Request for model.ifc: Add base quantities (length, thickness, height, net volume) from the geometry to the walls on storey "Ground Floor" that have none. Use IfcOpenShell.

First a look at what the model holds.

```python
import ifcopenshell
import ifcopenshell.util.element
import ifcopenshell.util.unit

model = ifcopenshell.open("model.ifc")
print(model.schema)
for unit_type in ("LENGTHUNIT", "AREAUNIT", "VOLUMEUNIT"):
    print(unit_type, ifcopenshell.util.unit.calculate_unit_scale(model, unit_type))
storey = next(s for s in model.by_type("IfcBuildingStorey") if s.Name == "Ground Floor")
walls = [e for e in ifcopenshell.util.element.get_decomposition(storey) if e.is_a("IfcWall")]
for e in sorted(walls, key=lambda e: e.id()):
    print(e.id(), e.is_a(), e.Name, list(ifcopenshell.util.element.get_psets(e, qtos_only=True)), sep=" | ")
```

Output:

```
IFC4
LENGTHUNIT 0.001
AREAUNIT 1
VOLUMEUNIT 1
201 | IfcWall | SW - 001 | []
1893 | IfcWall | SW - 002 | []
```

```python
import ifcopenshell
import ifcopenshell.api.pset
import ifcopenshell.geom
import ifcopenshell.util.element
import ifcopenshell.util.shape
import ifcopenshell.util.unit

model = ifcopenshell.open("model.ifc")
unit_scale = ifcopenshell.util.unit.calculate_unit_scale(model)
volume_scale = ifcopenshell.util.unit.calculate_unit_scale(model, "VOLUMEUNIT")
settings = ifcopenshell.geom.settings()

storey = next(s for s in model.by_type("IfcBuildingStorey") if s.Name == "Ground Floor")
walls = [e for e in ifcopenshell.util.element.get_decomposition(storey) if e.is_a("IfcWall")]

for e in sorted(walls, key=lambda e: e.id()):
    if ifcopenshell.util.element.get_psets(e, qtos_only=True, should_inherit=False):
        continue
    # Geometry comes back in metres, in the element's own axes.
    shape = ifcopenshell.geom.create_shape(settings, e)
    values = {
        "Length": ifcopenshell.util.shape.get_x(shape.geometry) / unit_scale,
        "Width": ifcopenshell.util.shape.get_y(shape.geometry) / unit_scale,
        "Height": ifcopenshell.util.shape.get_z(shape.geometry) / unit_scale,
        "NetVolume": ifcopenshell.util.shape.get_volume(shape.geometry) / volume_scale,
    }
    qto = ifcopenshell.api.pset.add_qto(model, product=e, name="Qto_WallBaseQuantities")
    ifcopenshell.api.pset.edit_qto(model, qto=qto, properties=values)
    print(e.id(), {k: round(v, 3) for k, v in values.items()})

model.write("model_v2.ifc")
```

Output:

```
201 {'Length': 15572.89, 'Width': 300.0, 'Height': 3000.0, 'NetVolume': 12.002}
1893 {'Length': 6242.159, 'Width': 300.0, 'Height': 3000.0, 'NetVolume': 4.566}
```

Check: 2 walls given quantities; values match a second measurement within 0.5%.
